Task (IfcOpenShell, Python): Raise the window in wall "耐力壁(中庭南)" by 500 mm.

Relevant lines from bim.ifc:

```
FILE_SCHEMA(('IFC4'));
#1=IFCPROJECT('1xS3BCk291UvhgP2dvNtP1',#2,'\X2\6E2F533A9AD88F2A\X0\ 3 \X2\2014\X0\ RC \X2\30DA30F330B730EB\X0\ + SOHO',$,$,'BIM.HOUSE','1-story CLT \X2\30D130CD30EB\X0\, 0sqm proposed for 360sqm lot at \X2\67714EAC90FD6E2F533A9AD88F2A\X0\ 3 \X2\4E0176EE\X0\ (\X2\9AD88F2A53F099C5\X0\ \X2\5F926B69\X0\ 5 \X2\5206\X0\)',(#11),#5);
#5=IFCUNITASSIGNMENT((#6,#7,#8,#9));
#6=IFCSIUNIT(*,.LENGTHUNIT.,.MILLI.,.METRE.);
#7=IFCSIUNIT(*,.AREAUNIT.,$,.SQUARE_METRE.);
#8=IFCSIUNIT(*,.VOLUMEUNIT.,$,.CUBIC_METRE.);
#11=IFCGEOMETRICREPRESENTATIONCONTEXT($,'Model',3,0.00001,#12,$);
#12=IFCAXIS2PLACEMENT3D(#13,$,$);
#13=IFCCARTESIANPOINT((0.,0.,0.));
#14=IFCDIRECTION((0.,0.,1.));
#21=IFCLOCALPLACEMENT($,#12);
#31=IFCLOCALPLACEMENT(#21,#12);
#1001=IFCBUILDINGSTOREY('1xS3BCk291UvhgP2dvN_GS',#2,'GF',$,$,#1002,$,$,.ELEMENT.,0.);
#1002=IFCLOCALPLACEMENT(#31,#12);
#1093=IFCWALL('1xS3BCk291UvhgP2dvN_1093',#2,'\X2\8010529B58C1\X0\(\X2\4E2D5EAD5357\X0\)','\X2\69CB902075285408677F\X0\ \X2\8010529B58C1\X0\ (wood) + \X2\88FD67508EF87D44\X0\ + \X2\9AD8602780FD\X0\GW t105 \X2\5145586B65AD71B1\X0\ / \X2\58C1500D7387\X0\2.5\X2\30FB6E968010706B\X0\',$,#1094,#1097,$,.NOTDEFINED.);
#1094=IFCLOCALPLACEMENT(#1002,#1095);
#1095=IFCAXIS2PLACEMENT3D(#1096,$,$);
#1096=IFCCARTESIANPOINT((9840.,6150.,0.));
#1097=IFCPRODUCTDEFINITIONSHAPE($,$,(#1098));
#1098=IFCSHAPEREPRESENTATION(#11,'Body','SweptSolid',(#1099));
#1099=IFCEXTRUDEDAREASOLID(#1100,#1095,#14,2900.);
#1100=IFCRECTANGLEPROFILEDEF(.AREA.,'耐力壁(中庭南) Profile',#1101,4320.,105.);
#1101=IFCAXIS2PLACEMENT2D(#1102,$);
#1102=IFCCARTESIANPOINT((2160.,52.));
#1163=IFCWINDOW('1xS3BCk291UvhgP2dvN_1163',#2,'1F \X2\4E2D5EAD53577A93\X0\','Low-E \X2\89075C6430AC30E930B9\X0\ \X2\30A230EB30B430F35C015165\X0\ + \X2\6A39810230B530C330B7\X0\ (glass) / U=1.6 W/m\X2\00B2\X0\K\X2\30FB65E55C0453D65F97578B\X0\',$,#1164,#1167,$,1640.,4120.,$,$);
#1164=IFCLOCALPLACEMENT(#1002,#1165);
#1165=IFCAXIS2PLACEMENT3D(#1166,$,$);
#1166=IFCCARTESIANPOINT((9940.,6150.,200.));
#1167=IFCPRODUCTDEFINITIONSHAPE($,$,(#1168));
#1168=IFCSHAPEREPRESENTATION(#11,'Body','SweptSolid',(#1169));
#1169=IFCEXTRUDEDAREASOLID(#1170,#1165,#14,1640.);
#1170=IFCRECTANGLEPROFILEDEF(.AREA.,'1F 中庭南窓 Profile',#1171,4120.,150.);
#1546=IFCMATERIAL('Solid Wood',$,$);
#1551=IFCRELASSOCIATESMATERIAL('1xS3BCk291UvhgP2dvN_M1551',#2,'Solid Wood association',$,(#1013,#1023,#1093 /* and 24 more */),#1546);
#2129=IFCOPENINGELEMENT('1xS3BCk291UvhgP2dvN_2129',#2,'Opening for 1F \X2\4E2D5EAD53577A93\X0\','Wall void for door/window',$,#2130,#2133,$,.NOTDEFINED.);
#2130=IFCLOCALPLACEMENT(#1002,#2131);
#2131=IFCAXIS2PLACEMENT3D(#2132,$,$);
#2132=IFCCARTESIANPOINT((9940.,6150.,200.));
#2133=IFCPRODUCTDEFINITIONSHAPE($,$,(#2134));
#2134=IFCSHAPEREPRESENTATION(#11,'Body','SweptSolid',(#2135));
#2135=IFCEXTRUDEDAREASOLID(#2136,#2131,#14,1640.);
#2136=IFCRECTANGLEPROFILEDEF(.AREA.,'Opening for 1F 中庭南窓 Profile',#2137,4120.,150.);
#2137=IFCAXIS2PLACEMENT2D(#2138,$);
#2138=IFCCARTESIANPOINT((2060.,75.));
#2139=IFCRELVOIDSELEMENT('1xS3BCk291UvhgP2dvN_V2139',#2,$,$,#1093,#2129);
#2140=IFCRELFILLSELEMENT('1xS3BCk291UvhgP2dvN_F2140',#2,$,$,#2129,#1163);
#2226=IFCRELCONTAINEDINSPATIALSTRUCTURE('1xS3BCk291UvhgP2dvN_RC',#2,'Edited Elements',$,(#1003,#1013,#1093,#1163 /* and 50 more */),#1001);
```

```python
import numpy as np
import ifcopenshell
import ifcopenshell.api.geometry
import ifcopenshell.util.placement
import ifcopenshell.util.unit

model = ifcopenshell.open("bim.ifc")
unit_scale = ifcopenshell.util.unit.calculate_unit_scale(model)

window = model.by_id(1163)
opening = window.FillsVoids[0].RelatingOpeningElement
dz = 500.0

shift = np.array([0.0, 0.0, dz])
# The window is not placed relative to its opening, so move both.
for product in (opening, window):
    matrix = ifcopenshell.util.placement.get_local_placement(product.ObjectPlacement)
    matrix[:3, 3] += shift
    ifcopenshell.api.geometry.edit_object_placement(model, product=product, matrix=matrix, is_si=False)

print(f"moved by {dz * unit_scale:+.3f} m")

model.write("bim-out.ifc")
```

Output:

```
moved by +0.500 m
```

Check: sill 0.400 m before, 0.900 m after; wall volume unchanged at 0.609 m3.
